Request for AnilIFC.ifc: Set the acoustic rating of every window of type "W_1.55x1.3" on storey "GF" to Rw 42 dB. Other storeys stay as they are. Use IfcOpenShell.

First a look at what the model holds.

```python
import ifcopenshell
import ifcopenshell.util.element

model = ifcopenshell.open("AnilIFC.ifc")
print(model.schema)
storey = next(s for s in model.by_type("IfcBuildingStorey") if s.Name == "GF")
windows = [e for e in ifcopenshell.util.element.get_decomposition(storey) if e.is_a("IfcWindow")]
seen = {}
for e in windows:
    element_type = ifcopenshell.util.element.get_type(e)
    key = (element_type.Name if element_type != e and element_type else None, ifcopenshell.util.element.get_pset(e, "Pset_WindowCommon", "AcousticRating"))
    seen[key] = seen.get(key, 0) + 1
for (name, value), count in sorted(seen.items(), key=str):
    print(count, "x", name, "|", value)
```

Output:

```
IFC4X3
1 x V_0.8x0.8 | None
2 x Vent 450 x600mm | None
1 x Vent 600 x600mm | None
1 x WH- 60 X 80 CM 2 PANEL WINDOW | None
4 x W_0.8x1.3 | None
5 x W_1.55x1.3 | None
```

```python
import ifcopenshell
import ifcopenshell.api.pset
import ifcopenshell.util.element

model = ifcopenshell.open("AnilIFC.ifc")

storey = next(s for s in model.by_type("IfcBuildingStorey") if s.Name == "GF")
windows = [e for e in ifcopenshell.util.element.get_decomposition(storey) if e.is_a("IfcWindow")]

count = 0
for e in windows:
    element_type = ifcopenshell.util.element.get_type(e)
    if element_type in (None, e) or element_type.Name != "W_1.55x1.3":
        continue
    # add_pset returns the element's existing set when there is one.
    pset = ifcopenshell.api.pset.add_pset(model, product=e, name="Pset_WindowCommon")
    ifcopenshell.api.pset.edit_pset(model, pset=pset, properties={"AcousticRating": "Rw 42 dB"})
    count += 1

print(count, "windows updated")

model.write("AnilIFC_v2.ifc")
```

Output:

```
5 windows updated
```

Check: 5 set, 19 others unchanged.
